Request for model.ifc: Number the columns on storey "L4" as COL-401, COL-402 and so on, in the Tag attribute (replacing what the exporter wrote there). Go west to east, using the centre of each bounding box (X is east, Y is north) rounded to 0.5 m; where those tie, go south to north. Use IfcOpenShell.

First a look at what the model holds.

```python
import ifcopenshell
import ifcopenshell.util.element
import ifcopenshell.util.placement

model = ifcopenshell.open("model.ifc")
print(model.schema)
storey = next(s for s in model.by_type("IfcBuildingStorey") if s.Name == "L4")
columns = [e for e in ifcopenshell.util.element.get_decomposition(storey) if e.is_a("IfcColumn")]
for e in sorted(columns, key=lambda e: e.id()):
    origin = ifcopenshell.util.placement.get_local_placement(e.ObjectPlacement)[:3, 3]
    print(e.id(), e.Tag, e.Name, origin.round(2) + 0.0, sep=" | ")
```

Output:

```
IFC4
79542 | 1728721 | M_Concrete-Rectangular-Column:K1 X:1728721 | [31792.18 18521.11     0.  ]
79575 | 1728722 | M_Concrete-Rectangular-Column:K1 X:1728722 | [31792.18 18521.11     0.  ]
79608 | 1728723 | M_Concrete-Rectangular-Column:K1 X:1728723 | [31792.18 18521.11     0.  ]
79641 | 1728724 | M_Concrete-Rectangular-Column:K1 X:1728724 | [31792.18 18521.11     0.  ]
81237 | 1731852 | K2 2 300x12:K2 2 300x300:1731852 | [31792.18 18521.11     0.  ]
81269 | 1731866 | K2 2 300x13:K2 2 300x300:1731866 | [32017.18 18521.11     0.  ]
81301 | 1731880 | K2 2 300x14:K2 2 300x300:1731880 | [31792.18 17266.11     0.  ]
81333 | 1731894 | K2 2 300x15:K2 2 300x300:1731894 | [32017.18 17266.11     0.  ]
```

```python
import ifcopenshell
import ifcopenshell.geom
import ifcopenshell.util.element
import ifcopenshell.util.shape

model = ifcopenshell.open("model.ifc")
settings = ifcopenshell.geom.settings()
settings.set("use-world-coords", True)


def centre(element):
    shape = ifcopenshell.geom.create_shape(settings, element)
    return ifcopenshell.util.shape.get_bbox_centroid(shape.geometry)


storey = next(s for s in model.by_type("IfcBuildingStorey") if s.Name == "L4")
columns = [e for e in ifcopenshell.util.element.get_decomposition(storey) if e.is_a("IfcColumn")]

# Insertion points can sit at a corner or the storey origin, so sort by the geometry (in metres).
centres = {e: centre(e) for e in columns}
columns.sort(key=lambda e: (round(centres[e][0] / 0.5), centres[e][1]))

for i, e in enumerate(columns, start=1):
    number = f"COL-4{i:02d}"
    e.Tag = number
    print(e.id(), number)

model.write("model_edited.ifc")
```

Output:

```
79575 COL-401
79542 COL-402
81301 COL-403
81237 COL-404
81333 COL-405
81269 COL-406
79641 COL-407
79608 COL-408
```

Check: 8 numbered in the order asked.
